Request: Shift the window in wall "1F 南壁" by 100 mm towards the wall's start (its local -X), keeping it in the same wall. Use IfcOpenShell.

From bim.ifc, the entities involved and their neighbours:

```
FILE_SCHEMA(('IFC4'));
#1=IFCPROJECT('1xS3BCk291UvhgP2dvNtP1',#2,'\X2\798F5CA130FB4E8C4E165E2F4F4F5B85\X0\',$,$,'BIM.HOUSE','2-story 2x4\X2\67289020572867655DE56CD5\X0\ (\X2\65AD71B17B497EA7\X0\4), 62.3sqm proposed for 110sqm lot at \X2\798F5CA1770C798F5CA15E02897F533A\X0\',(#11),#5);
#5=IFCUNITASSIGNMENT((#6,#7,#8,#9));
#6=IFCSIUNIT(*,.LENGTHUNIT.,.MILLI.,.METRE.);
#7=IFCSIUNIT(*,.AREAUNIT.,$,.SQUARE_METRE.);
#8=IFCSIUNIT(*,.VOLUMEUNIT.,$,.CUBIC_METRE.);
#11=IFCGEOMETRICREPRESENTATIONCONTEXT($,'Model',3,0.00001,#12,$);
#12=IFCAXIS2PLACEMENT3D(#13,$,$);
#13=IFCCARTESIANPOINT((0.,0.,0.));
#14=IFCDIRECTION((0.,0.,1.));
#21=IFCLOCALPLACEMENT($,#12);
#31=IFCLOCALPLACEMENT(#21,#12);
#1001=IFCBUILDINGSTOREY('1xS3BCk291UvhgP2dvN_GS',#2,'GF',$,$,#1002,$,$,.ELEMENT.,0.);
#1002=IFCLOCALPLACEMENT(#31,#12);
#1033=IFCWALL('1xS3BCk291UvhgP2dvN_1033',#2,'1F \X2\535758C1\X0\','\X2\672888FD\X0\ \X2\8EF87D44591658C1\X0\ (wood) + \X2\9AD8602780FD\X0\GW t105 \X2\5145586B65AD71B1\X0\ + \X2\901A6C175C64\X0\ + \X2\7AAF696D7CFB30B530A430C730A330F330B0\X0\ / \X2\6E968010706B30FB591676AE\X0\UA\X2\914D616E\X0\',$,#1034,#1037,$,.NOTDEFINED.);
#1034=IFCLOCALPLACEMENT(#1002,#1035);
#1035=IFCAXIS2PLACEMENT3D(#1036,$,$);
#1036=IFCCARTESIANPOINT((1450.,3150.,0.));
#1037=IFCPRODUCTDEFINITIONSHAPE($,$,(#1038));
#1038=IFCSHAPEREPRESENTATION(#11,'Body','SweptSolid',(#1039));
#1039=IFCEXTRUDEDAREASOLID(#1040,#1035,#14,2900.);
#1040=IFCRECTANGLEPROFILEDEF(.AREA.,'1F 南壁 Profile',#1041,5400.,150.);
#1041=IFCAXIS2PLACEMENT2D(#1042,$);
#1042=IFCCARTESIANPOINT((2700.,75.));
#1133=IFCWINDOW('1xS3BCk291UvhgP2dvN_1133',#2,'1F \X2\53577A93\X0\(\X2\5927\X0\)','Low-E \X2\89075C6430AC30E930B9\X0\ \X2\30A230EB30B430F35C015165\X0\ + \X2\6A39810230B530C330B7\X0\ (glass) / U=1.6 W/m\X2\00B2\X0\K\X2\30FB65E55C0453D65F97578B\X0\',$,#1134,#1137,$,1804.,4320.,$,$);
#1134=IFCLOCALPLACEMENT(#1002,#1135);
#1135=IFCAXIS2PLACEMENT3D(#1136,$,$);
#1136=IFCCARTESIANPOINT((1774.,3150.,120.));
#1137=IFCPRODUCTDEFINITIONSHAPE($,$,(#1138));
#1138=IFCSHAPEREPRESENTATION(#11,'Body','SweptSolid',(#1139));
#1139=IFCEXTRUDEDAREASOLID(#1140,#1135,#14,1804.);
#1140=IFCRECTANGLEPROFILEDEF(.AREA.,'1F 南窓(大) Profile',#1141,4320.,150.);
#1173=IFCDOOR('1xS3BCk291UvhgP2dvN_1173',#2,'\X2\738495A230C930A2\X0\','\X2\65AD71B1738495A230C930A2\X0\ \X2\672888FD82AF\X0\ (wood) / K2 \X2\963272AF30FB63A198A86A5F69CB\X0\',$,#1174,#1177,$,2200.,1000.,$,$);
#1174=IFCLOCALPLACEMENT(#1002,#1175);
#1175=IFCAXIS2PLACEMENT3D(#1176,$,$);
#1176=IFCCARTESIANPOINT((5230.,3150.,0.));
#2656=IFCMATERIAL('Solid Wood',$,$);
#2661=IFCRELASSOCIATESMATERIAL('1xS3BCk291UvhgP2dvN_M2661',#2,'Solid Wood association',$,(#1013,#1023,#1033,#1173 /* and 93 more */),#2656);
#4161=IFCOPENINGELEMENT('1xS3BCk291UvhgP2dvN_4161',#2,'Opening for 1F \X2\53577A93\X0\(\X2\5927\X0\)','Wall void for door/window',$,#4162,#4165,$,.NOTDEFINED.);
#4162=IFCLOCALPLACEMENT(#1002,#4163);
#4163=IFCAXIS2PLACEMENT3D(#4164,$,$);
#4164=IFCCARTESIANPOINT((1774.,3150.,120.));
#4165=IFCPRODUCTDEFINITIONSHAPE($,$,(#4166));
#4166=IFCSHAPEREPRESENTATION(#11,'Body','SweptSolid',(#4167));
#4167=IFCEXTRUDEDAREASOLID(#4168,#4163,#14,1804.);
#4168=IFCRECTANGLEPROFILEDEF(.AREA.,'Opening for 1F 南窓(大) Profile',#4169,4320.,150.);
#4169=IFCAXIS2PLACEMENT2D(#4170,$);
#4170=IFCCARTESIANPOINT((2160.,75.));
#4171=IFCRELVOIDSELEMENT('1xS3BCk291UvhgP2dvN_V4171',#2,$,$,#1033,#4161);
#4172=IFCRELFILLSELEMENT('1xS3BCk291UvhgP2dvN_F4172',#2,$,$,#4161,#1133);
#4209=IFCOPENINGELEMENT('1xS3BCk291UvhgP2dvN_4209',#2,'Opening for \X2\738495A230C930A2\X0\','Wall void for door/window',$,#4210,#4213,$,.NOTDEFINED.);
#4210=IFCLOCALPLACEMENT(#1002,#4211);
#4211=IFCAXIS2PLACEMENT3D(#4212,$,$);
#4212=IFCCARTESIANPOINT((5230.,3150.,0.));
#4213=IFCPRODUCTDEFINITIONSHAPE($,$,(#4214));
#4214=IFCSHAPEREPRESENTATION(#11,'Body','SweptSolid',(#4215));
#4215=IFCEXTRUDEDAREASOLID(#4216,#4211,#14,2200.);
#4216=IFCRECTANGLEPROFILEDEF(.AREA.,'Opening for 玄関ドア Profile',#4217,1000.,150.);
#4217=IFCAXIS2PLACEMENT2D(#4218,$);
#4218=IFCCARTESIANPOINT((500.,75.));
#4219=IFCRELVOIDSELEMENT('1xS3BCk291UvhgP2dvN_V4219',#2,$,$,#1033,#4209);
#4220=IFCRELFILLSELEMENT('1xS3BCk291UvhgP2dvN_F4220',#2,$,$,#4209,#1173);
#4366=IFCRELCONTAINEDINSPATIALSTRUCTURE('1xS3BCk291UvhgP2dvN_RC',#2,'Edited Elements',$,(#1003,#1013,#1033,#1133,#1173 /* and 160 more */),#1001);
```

```python
import ifcopenshell
import ifcopenshell.api.geometry
import ifcopenshell.util.placement
import ifcopenshell.util.unit

model = ifcopenshell.open("bim.ifc")
unit_scale = ifcopenshell.util.unit.calculate_unit_scale(model)

window = model.by_id(1133)
opening = window.FillsVoids[0].RelatingOpeningElement
wall = opening.VoidsElements[0].RelatingBuildingElement

wall_matrix = ifcopenshell.util.placement.get_local_placement(wall.ObjectPlacement)
shift = wall_matrix[:3, 0] * -0.1 / unit_scale
before = ifcopenshell.util.placement.get_local_placement(window.ObjectPlacement)[:3, 3].copy()

# The window is not placed relative to its opening, so move both.
for product in (opening, window):
    matrix = ifcopenshell.util.placement.get_local_placement(product.ObjectPlacement)
    matrix[:3, 3] += shift
    ifcopenshell.api.geometry.edit_object_placement(model, product=product, matrix=matrix, is_si=False)

after = ifcopenshell.util.placement.get_local_placement(window.ObjectPlacement)[:3, 3]
print("window moved by", (after - before).round(3) + 0.0)

model.write("bim-out.ifc")
```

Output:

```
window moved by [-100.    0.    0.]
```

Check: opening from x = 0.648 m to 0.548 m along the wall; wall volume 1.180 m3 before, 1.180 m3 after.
